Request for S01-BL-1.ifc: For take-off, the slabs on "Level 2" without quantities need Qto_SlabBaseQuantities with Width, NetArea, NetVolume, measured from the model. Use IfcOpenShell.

First a look at what the model holds.

```python
import ifcopenshell
import ifcopenshell.util.element
import ifcopenshell.util.unit

model = ifcopenshell.open("S01-BL-1.ifc")
print(model.schema)
for unit_type in ("LENGTHUNIT", "AREAUNIT", "VOLUMEUNIT"):
    print(unit_type, ifcopenshell.util.unit.calculate_unit_scale(model, unit_type))
storey = next(s for s in model.by_type("IfcBuildingStorey") if s.Name == "Level 2")
slabs = [e for e in ifcopenshell.util.element.get_decomposition(storey) if e.is_a("IfcSlab")]
for e in sorted(slabs, key=lambda e: e.id()):
    print(e.id(), e.is_a(), e.Name, list(ifcopenshell.util.element.get_psets(e, qtos_only=True)), sep=" | ")
```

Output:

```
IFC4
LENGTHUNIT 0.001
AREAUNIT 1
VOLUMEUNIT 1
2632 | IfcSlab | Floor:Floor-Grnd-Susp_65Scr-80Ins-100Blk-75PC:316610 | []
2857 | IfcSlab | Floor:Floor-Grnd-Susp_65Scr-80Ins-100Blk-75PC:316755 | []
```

```python
import ifcopenshell
import ifcopenshell.api.pset
import ifcopenshell.geom
import ifcopenshell.util.element
import ifcopenshell.util.shape
import ifcopenshell.util.unit

model = ifcopenshell.open("S01-BL-1.ifc")
unit_scale = ifcopenshell.util.unit.calculate_unit_scale(model)
area_scale = ifcopenshell.util.unit.calculate_unit_scale(model, "AREAUNIT")
volume_scale = ifcopenshell.util.unit.calculate_unit_scale(model, "VOLUMEUNIT")
settings = ifcopenshell.geom.settings()

storey = next(s for s in model.by_type("IfcBuildingStorey") if s.Name == "Level 2")
slabs = [e for e in ifcopenshell.util.element.get_decomposition(storey) if e.is_a("IfcSlab")]

for e in sorted(slabs, key=lambda e: e.id()):
    if ifcopenshell.util.element.get_psets(e, qtos_only=True, should_inherit=False):
        continue
    # Geometry comes back in metres, in the element's own axes.
    shape = ifcopenshell.geom.create_shape(settings, e)
    values = {
        "Width": ifcopenshell.util.shape.get_z(shape.geometry) / unit_scale,
        "NetArea": ifcopenshell.util.shape.get_footprint_area(shape.geometry) / area_scale,
        "NetVolume": ifcopenshell.util.shape.get_volume(shape.geometry) / volume_scale,
    }
    qto = ifcopenshell.api.pset.add_qto(model, product=e, name="Qto_SlabBaseQuantities")
    ifcopenshell.api.pset.edit_qto(model, qto=qto, properties=values)
    print(e.id(), {k: round(v, 3) for k, v in values.items()})

model.write("S01-BL-1_updated.ifc")
```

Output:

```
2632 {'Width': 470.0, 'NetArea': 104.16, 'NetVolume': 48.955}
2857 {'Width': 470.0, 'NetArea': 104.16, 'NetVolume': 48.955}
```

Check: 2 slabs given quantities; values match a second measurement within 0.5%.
